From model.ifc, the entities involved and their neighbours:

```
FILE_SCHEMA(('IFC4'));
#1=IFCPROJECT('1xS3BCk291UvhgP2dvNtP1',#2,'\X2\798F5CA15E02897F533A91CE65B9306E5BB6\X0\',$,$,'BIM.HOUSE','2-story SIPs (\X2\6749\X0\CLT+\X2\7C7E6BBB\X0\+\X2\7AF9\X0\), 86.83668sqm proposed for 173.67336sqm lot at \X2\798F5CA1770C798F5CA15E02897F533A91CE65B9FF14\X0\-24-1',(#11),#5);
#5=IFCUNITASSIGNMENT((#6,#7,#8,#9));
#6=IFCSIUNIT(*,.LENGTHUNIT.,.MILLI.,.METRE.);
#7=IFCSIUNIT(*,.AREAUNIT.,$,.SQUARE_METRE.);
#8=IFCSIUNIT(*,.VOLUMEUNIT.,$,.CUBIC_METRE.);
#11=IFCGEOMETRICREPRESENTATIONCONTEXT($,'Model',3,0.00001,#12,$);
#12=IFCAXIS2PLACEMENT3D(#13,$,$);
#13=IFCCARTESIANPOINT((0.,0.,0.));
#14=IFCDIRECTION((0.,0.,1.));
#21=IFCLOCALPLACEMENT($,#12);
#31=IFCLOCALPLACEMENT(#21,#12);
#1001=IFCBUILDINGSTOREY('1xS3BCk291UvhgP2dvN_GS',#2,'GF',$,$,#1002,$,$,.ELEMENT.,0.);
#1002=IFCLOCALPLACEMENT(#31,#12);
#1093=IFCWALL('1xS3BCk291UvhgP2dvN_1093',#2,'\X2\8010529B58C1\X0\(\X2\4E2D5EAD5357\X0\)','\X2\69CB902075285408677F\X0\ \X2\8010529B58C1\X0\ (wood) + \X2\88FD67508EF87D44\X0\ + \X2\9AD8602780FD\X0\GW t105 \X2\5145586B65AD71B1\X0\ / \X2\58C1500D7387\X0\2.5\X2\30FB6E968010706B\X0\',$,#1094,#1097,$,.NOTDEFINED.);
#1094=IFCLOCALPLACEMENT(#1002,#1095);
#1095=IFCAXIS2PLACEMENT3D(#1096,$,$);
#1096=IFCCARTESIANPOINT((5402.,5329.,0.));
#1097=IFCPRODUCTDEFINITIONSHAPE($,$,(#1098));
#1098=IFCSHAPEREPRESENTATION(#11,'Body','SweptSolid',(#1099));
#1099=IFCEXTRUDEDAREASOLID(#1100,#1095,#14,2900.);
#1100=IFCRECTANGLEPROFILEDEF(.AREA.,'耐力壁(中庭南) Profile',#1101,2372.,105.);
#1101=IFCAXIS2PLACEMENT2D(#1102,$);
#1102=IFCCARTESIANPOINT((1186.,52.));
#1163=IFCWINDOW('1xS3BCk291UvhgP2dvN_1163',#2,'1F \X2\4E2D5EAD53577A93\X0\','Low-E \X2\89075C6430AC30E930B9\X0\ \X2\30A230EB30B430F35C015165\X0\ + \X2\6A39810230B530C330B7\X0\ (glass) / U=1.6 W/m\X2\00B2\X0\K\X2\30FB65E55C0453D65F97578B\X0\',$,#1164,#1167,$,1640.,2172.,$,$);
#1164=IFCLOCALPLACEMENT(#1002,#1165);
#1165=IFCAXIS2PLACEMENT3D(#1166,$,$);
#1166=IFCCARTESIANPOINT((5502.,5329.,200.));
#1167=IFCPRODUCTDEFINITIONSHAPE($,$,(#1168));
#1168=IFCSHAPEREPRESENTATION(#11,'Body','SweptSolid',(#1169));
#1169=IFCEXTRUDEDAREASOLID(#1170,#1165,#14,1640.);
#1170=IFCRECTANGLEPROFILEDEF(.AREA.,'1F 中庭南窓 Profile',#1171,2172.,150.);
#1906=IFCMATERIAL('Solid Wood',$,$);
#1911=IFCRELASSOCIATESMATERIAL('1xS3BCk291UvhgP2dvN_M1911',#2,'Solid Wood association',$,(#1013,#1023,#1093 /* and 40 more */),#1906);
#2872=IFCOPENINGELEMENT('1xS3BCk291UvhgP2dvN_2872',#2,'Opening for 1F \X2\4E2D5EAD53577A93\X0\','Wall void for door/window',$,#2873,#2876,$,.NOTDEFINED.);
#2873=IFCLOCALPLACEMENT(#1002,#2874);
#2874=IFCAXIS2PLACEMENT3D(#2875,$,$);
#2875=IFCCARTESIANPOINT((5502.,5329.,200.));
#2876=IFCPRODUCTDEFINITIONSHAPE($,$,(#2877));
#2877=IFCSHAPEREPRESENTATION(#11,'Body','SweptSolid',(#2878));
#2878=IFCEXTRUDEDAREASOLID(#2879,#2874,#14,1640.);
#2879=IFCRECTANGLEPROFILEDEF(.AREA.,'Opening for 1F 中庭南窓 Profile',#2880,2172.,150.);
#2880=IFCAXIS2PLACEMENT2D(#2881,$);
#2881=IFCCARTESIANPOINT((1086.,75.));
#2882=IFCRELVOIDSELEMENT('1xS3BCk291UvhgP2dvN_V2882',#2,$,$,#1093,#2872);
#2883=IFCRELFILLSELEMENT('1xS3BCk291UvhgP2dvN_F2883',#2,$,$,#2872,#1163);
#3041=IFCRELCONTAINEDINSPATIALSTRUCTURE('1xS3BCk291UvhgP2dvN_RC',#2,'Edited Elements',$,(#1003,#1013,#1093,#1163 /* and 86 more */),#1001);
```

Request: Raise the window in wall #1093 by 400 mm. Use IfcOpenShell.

```python
import numpy as np
import ifcopenshell
import ifcopenshell.api.geometry
import ifcopenshell.util.placement
import ifcopenshell.util.unit

model = ifcopenshell.open("model.ifc")
unit_scale = ifcopenshell.util.unit.calculate_unit_scale(model)

window = model.by_guid("1xS3BCk291UvhgP2dvN_1163")
opening = window.FillsVoids[0].RelatingOpeningElement
dz = 400.0

shift = np.array([0.0, 0.0, dz])
# The window is not placed relative to its opening, so move both.
for product in (opening, window):
    matrix = ifcopenshell.util.placement.get_local_placement(product.ObjectPlacement)
    matrix[:3, 3] += shift
    ifcopenshell.api.geometry.edit_object_placement(model, product=product, matrix=matrix, is_si=False)

print(f"moved by {dz * unit_scale:+.3f} m")

model.write("model_rev.ifc")
```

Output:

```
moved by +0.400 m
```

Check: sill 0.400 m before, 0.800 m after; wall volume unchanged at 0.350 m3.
